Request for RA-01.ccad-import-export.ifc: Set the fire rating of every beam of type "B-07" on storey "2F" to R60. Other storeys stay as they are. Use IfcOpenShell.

First a look at what the model holds.

```python
import ifcopenshell
import ifcopenshell.util.element

model = ifcopenshell.open("RA-01.ccad-import-export.ifc")
print(model.schema)
storey = next(s for s in model.by_type("IfcBuildingStorey") if s.Name == "2F")
beams = [e for e in ifcopenshell.util.element.get_decomposition(storey) if e.is_a("IfcBeam")]
seen = {}
for e in beams:
    element_type = ifcopenshell.util.element.get_type(e)
    key = (element_type.Name if element_type != e and element_type else None, ifcopenshell.util.element.get_pset(e, "Pset_BeamCommon", "FireRating"))
    seen[key] = seen.get(key, 0) + 1
for (name, value), count in sorted(seen.items(), key=str):
    print(count, "x", name, "|", value)
```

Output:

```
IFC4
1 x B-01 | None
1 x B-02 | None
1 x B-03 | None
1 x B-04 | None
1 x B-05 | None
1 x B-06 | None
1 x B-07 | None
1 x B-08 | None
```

```python
import ifcopenshell
import ifcopenshell.api.pset
import ifcopenshell.util.element

model = ifcopenshell.open("RA-01.ccad-import-export.ifc")

storey = next(s for s in model.by_type("IfcBuildingStorey") if s.Name == "2F")
beams = [e for e in ifcopenshell.util.element.get_decomposition(storey) if e.is_a("IfcBeam")]

count = 0
for e in beams:
    element_type = ifcopenshell.util.element.get_type(e)
    if element_type in (None, e) or element_type.Name != "B-07":
        continue
    found = ifcopenshell.util.element.get_pset(e, "Pset_BeamCommon", should_inherit=False)
    if found:
        pset = model.by_id(found["id"])
        if len(ifcopenshell.util.element.get_elements_by_pset(pset)) > 1:
            pset = ifcopenshell.api.pset.unshare_pset(model, products=[e], pset=pset)[0]
    else:
        pset = ifcopenshell.api.pset.add_pset(model, product=e, name="Pset_BeamCommon")
    ifcopenshell.api.pset.edit_pset(model, pset=pset, properties={"FireRating": "R60"})
    count += 1

print(count, "beams updated")

model.write("RA-01.ccad-import-export_edited.ifc")
```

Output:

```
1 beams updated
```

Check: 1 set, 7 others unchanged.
